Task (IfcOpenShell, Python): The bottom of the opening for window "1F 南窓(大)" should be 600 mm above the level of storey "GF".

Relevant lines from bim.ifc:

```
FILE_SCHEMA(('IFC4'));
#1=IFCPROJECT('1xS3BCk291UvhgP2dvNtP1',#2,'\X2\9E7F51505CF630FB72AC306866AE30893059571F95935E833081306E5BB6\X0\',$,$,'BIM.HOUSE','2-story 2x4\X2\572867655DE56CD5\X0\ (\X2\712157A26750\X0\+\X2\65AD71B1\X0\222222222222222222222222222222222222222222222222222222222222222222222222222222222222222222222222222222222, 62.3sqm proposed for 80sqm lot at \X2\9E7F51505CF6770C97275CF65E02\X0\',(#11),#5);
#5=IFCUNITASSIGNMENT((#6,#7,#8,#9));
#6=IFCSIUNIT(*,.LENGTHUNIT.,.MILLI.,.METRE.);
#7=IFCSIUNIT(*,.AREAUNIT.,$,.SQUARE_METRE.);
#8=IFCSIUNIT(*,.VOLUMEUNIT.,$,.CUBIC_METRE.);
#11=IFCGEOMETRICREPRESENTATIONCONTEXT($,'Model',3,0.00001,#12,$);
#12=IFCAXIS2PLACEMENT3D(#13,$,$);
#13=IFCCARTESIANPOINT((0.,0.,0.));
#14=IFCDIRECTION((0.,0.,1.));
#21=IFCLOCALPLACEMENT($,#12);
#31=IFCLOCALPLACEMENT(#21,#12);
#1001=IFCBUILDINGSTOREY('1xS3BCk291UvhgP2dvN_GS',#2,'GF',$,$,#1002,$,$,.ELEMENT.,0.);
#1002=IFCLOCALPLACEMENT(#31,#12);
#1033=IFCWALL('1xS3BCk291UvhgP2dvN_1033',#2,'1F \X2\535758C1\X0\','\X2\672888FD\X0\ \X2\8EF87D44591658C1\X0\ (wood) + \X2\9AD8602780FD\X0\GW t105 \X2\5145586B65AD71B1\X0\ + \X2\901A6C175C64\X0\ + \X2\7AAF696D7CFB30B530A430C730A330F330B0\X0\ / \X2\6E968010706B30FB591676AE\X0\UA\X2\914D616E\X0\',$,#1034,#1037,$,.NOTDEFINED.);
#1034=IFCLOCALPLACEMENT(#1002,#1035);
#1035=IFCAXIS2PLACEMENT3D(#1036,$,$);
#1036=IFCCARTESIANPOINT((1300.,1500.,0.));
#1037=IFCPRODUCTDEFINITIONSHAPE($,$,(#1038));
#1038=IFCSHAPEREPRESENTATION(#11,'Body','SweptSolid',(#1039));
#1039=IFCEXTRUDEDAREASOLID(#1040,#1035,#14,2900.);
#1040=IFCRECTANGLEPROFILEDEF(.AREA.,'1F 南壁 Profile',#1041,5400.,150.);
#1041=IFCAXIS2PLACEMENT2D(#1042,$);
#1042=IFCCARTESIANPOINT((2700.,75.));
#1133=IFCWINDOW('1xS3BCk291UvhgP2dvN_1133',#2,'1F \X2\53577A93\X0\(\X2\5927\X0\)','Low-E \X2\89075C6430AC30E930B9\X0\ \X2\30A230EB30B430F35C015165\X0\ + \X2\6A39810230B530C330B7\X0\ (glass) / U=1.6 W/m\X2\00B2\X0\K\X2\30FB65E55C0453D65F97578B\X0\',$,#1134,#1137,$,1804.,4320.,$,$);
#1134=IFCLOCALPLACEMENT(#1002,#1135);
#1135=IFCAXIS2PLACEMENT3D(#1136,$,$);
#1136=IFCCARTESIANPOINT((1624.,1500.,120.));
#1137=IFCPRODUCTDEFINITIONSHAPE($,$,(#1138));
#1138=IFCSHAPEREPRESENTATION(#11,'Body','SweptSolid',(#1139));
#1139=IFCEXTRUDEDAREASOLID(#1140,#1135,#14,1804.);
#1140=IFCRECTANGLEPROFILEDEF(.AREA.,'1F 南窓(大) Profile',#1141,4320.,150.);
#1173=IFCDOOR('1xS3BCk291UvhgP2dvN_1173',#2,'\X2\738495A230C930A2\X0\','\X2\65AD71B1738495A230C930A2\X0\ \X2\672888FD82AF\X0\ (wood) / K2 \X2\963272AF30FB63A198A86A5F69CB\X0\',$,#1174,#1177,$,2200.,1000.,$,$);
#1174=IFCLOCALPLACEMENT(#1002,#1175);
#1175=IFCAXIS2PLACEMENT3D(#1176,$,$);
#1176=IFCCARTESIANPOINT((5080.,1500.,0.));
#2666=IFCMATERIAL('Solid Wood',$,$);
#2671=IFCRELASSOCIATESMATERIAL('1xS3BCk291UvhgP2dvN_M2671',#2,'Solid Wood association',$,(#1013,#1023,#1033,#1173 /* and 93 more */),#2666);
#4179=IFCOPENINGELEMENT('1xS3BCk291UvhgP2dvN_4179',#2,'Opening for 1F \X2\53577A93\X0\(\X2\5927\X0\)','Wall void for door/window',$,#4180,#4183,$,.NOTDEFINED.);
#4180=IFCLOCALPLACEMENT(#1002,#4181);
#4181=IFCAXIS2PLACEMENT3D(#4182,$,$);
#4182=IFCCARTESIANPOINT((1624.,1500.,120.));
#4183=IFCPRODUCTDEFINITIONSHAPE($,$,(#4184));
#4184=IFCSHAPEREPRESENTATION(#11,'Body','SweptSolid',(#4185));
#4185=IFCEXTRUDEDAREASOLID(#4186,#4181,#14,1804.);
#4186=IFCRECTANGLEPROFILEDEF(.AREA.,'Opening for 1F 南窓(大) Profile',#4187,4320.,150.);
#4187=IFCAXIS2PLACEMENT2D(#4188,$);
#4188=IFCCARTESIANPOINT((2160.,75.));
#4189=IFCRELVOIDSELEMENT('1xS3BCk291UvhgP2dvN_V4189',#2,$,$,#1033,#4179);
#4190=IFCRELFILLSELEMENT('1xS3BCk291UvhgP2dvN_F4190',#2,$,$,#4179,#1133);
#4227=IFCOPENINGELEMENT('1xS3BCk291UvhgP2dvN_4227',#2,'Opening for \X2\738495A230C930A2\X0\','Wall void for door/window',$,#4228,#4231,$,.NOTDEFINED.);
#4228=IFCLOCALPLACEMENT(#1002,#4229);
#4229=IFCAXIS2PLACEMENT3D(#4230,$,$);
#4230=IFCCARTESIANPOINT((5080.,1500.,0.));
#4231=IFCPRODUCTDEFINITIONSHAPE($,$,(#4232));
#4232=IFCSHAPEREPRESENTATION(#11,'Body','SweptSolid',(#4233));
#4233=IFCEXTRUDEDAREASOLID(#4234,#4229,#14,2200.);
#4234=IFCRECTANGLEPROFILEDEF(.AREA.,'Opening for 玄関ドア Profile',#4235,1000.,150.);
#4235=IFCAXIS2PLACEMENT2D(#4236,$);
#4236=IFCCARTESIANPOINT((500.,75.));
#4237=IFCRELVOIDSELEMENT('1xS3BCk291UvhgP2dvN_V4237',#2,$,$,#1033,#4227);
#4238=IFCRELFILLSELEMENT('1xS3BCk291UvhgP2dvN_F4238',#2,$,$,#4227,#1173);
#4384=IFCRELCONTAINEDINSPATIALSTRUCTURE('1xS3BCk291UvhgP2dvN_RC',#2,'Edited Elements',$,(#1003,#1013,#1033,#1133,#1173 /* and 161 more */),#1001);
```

```python
import numpy as np
import ifcopenshell
import ifcopenshell.api.geometry
import ifcopenshell.geom
import ifcopenshell.util.element
import ifcopenshell.util.placement
import ifcopenshell.util.shape
import ifcopenshell.util.unit

model = ifcopenshell.open("bim.ifc")
unit_scale = ifcopenshell.util.unit.calculate_unit_scale(model)

window = model.by_guid("1xS3BCk291UvhgP2dvN_1133")
opening = window.FillsVoids[0].RelatingOpeningElement
storey = ifcopenshell.util.element.get_container(window, ifc_class="IfcBuildingStorey")
level = ifcopenshell.util.placement.get_local_placement(storey.ObjectPlacement)[2, 3]

# The opening's origin need not be at the sill, so measure its lowest point.
shape = ifcopenshell.geom.create_shape(ifcopenshell.geom.settings(), opening)
bottom = ifcopenshell.util.shape.get_shape_bottom_elevation(shape, shape.geometry) / unit_scale
dz = level + 0.6 / unit_scale - bottom

shift = np.array([0.0, 0.0, dz])
# The window is not placed relative to its opening, so move both.
for product in (opening, window):
    matrix = ifcopenshell.util.placement.get_local_placement(product.ObjectPlacement)
    matrix[:3, 3] += shift
    ifcopenshell.api.geometry.edit_object_placement(model, product=product, matrix=matrix, is_si=False)

print(f"moved by {dz * unit_scale:+.3f} m")

model.write("bim_rev.ifc")
```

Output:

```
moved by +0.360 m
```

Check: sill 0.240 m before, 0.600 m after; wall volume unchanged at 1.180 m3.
